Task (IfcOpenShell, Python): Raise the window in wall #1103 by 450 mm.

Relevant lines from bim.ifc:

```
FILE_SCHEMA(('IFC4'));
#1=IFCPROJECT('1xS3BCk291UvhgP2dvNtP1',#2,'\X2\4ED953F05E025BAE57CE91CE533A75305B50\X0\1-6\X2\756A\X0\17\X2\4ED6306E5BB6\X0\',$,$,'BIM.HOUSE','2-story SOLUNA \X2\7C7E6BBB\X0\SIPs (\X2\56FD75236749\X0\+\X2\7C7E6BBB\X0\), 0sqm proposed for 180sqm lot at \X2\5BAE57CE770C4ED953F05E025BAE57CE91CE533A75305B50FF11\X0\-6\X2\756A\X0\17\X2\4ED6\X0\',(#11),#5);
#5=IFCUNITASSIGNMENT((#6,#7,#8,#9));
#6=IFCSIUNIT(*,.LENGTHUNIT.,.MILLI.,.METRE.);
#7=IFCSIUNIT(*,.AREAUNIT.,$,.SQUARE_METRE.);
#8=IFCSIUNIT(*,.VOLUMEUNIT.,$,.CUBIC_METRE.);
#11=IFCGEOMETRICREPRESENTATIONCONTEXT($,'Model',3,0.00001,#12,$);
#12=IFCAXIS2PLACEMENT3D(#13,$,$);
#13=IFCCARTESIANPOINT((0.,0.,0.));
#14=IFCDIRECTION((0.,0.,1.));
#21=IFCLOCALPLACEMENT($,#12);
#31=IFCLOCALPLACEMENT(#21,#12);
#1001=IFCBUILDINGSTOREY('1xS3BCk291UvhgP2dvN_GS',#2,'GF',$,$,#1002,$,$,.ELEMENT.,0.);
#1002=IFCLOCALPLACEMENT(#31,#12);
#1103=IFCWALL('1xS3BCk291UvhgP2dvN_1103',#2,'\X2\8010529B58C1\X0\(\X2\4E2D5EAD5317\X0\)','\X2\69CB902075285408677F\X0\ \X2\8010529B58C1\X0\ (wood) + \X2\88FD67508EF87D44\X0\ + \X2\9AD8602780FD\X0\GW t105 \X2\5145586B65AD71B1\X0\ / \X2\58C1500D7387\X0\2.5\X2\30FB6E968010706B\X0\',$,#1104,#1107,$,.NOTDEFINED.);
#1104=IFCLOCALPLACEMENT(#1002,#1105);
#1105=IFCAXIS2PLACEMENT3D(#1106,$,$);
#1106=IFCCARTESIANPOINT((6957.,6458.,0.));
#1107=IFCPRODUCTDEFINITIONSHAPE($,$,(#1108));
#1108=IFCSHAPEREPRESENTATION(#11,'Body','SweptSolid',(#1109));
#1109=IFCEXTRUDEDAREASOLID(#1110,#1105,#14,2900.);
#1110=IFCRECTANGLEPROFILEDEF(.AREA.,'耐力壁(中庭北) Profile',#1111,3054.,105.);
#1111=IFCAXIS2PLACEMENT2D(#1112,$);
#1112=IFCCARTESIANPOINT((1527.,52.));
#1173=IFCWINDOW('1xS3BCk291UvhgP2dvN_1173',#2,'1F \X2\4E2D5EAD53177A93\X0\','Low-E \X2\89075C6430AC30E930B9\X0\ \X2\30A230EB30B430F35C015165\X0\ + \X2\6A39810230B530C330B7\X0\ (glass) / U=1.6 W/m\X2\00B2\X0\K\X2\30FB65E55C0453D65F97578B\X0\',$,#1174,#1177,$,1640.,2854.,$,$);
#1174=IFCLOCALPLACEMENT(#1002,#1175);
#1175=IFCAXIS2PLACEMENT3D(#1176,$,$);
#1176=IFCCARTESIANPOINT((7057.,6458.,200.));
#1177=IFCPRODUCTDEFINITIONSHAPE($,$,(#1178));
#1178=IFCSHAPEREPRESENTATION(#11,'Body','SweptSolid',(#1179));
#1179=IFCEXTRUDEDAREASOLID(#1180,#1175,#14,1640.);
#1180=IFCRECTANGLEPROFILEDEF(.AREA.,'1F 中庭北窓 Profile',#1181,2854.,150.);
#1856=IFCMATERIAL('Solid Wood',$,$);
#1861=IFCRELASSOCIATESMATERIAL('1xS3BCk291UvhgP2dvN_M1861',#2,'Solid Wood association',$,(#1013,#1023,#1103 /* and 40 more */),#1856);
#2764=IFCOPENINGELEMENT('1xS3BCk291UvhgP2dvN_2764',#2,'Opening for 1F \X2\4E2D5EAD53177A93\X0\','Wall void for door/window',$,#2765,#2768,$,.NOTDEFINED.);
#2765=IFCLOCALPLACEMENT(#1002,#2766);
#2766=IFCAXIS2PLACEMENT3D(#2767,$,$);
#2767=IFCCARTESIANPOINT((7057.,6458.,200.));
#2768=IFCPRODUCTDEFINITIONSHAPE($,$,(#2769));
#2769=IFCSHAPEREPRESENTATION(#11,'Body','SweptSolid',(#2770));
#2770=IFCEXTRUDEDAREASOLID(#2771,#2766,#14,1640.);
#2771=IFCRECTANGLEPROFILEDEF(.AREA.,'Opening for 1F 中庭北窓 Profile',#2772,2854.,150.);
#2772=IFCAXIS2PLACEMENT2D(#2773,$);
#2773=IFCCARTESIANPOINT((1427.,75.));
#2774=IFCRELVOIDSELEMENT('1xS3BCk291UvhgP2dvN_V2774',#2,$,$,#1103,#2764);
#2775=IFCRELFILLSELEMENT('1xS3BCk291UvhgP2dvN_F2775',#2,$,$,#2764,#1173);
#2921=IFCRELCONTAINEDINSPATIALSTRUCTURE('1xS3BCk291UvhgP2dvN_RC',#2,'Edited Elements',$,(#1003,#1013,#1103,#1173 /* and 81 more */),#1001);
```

```python
import numpy as np
import ifcopenshell
import ifcopenshell.api.geometry
import ifcopenshell.util.placement
import ifcopenshell.util.unit

model = ifcopenshell.open("bim.ifc")
unit_scale = ifcopenshell.util.unit.calculate_unit_scale(model)

window = model.by_guid("1xS3BCk291UvhgP2dvN_1173")
opening = window.FillsVoids[0].RelatingOpeningElement
dz = 0.45 / unit_scale

shift = np.array([0.0, 0.0, dz])
# The window is not placed relative to its opening, so move both.
for product in (opening, window):
    matrix = ifcopenshell.util.placement.get_local_placement(product.ObjectPlacement)
    matrix[:3, 3] += shift
    ifcopenshell.api.geometry.edit_object_placement(model, product=product, matrix=matrix, is_si=False)

print(f"moved by {dz * unit_scale:+.3f} m")

model.write("bim_updated.ifc")
```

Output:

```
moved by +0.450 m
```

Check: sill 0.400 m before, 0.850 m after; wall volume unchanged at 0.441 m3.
